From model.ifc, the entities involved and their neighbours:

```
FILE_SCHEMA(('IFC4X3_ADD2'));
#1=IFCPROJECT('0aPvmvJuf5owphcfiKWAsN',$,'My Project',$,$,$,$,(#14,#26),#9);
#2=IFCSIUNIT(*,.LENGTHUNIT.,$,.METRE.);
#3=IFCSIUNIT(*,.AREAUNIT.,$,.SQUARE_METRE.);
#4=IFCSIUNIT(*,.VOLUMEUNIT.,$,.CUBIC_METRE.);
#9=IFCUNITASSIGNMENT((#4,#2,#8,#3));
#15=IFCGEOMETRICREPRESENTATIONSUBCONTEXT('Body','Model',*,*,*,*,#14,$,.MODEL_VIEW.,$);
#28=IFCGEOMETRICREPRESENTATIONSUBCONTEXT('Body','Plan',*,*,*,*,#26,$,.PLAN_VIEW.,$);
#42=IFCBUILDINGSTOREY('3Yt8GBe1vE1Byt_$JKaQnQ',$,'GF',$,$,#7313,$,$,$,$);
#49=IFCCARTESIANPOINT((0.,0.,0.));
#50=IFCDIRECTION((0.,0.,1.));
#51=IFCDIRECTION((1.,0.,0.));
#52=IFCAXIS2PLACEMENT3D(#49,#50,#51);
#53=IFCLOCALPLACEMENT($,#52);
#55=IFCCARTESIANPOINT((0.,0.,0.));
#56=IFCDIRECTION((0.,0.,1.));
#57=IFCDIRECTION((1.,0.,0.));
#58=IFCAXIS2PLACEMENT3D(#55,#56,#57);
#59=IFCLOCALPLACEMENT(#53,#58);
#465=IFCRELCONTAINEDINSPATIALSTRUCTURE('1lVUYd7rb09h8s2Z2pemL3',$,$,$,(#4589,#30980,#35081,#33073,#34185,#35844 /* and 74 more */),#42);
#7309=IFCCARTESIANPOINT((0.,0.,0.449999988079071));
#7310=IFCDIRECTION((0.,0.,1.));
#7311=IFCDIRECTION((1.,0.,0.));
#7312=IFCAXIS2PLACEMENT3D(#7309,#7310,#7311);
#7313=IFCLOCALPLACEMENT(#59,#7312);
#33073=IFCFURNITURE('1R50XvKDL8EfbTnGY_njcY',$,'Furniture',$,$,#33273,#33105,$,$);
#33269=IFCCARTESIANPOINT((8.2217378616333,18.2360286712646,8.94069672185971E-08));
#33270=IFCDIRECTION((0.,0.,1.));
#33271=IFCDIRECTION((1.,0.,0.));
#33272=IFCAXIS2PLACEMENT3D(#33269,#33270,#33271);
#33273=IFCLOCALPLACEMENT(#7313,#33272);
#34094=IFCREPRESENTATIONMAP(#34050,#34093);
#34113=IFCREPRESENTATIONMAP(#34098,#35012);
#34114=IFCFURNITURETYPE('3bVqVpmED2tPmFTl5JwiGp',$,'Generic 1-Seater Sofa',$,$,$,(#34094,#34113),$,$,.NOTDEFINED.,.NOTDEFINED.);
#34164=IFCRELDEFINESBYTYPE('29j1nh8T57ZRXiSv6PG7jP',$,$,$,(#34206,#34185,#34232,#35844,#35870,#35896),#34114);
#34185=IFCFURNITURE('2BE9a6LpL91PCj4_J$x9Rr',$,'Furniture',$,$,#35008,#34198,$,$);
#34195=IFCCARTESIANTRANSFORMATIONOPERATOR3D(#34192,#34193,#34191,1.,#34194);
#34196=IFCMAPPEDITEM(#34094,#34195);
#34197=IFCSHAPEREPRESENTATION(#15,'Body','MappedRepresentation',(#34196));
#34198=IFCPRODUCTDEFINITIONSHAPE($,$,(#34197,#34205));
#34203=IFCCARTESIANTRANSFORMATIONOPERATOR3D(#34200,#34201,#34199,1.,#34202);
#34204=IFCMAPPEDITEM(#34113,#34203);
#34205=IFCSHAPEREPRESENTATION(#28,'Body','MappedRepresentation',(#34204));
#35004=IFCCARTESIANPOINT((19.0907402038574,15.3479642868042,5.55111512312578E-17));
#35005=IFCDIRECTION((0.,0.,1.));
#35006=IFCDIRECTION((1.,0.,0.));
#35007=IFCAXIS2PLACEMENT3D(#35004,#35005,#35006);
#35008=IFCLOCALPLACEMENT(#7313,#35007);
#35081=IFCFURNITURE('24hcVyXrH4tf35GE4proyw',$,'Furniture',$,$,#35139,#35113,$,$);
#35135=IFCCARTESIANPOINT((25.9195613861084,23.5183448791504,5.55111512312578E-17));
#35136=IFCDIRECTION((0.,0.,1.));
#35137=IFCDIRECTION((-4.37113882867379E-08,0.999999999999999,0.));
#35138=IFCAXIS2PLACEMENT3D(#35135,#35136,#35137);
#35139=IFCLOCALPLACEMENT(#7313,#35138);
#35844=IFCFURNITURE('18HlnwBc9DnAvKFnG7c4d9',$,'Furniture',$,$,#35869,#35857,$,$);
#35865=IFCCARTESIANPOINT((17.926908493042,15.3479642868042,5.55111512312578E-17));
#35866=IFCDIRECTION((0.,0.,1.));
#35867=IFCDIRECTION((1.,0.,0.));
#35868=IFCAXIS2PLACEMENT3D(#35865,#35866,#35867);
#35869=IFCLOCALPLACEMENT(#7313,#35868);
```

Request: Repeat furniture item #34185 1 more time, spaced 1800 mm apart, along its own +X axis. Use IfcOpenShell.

```python
import ifcopenshell
import ifcopenshell.api.geometry
import ifcopenshell.api.root
import ifcopenshell.util.element
import ifcopenshell.util.placement
import ifcopenshell.util.unit

model = ifcopenshell.open("model.ifc")
unit_scale = ifcopenshell.util.unit.calculate_unit_scale(model)

source = model.by_guid("2BE9a6LpL91PCj4_J$x9Rr")
base = ifcopenshell.util.placement.get_local_placement(source.ObjectPlacement)
step = base[:3, 0] * 1.8 / unit_scale

for i in range(1, 2):
    copy = ifcopenshell.api.root.copy_class(model, product=source)
    copy.Representation = ifcopenshell.util.element.copy_deep(
        model, source.Representation, exclude=["IfcGeometricRepresentationContext", "IfcRepresentationMap"]
    )
    matrix = base.copy()
    matrix[:3, 3] += i * step
    print("added at", matrix[:3, 3].round(3) + 0.0)
    ifcopenshell.api.geometry.edit_object_placement(model, product=copy, matrix=matrix, is_si=False)

model.write("model_updated.ifc")
```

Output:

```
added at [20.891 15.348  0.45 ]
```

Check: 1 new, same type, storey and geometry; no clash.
